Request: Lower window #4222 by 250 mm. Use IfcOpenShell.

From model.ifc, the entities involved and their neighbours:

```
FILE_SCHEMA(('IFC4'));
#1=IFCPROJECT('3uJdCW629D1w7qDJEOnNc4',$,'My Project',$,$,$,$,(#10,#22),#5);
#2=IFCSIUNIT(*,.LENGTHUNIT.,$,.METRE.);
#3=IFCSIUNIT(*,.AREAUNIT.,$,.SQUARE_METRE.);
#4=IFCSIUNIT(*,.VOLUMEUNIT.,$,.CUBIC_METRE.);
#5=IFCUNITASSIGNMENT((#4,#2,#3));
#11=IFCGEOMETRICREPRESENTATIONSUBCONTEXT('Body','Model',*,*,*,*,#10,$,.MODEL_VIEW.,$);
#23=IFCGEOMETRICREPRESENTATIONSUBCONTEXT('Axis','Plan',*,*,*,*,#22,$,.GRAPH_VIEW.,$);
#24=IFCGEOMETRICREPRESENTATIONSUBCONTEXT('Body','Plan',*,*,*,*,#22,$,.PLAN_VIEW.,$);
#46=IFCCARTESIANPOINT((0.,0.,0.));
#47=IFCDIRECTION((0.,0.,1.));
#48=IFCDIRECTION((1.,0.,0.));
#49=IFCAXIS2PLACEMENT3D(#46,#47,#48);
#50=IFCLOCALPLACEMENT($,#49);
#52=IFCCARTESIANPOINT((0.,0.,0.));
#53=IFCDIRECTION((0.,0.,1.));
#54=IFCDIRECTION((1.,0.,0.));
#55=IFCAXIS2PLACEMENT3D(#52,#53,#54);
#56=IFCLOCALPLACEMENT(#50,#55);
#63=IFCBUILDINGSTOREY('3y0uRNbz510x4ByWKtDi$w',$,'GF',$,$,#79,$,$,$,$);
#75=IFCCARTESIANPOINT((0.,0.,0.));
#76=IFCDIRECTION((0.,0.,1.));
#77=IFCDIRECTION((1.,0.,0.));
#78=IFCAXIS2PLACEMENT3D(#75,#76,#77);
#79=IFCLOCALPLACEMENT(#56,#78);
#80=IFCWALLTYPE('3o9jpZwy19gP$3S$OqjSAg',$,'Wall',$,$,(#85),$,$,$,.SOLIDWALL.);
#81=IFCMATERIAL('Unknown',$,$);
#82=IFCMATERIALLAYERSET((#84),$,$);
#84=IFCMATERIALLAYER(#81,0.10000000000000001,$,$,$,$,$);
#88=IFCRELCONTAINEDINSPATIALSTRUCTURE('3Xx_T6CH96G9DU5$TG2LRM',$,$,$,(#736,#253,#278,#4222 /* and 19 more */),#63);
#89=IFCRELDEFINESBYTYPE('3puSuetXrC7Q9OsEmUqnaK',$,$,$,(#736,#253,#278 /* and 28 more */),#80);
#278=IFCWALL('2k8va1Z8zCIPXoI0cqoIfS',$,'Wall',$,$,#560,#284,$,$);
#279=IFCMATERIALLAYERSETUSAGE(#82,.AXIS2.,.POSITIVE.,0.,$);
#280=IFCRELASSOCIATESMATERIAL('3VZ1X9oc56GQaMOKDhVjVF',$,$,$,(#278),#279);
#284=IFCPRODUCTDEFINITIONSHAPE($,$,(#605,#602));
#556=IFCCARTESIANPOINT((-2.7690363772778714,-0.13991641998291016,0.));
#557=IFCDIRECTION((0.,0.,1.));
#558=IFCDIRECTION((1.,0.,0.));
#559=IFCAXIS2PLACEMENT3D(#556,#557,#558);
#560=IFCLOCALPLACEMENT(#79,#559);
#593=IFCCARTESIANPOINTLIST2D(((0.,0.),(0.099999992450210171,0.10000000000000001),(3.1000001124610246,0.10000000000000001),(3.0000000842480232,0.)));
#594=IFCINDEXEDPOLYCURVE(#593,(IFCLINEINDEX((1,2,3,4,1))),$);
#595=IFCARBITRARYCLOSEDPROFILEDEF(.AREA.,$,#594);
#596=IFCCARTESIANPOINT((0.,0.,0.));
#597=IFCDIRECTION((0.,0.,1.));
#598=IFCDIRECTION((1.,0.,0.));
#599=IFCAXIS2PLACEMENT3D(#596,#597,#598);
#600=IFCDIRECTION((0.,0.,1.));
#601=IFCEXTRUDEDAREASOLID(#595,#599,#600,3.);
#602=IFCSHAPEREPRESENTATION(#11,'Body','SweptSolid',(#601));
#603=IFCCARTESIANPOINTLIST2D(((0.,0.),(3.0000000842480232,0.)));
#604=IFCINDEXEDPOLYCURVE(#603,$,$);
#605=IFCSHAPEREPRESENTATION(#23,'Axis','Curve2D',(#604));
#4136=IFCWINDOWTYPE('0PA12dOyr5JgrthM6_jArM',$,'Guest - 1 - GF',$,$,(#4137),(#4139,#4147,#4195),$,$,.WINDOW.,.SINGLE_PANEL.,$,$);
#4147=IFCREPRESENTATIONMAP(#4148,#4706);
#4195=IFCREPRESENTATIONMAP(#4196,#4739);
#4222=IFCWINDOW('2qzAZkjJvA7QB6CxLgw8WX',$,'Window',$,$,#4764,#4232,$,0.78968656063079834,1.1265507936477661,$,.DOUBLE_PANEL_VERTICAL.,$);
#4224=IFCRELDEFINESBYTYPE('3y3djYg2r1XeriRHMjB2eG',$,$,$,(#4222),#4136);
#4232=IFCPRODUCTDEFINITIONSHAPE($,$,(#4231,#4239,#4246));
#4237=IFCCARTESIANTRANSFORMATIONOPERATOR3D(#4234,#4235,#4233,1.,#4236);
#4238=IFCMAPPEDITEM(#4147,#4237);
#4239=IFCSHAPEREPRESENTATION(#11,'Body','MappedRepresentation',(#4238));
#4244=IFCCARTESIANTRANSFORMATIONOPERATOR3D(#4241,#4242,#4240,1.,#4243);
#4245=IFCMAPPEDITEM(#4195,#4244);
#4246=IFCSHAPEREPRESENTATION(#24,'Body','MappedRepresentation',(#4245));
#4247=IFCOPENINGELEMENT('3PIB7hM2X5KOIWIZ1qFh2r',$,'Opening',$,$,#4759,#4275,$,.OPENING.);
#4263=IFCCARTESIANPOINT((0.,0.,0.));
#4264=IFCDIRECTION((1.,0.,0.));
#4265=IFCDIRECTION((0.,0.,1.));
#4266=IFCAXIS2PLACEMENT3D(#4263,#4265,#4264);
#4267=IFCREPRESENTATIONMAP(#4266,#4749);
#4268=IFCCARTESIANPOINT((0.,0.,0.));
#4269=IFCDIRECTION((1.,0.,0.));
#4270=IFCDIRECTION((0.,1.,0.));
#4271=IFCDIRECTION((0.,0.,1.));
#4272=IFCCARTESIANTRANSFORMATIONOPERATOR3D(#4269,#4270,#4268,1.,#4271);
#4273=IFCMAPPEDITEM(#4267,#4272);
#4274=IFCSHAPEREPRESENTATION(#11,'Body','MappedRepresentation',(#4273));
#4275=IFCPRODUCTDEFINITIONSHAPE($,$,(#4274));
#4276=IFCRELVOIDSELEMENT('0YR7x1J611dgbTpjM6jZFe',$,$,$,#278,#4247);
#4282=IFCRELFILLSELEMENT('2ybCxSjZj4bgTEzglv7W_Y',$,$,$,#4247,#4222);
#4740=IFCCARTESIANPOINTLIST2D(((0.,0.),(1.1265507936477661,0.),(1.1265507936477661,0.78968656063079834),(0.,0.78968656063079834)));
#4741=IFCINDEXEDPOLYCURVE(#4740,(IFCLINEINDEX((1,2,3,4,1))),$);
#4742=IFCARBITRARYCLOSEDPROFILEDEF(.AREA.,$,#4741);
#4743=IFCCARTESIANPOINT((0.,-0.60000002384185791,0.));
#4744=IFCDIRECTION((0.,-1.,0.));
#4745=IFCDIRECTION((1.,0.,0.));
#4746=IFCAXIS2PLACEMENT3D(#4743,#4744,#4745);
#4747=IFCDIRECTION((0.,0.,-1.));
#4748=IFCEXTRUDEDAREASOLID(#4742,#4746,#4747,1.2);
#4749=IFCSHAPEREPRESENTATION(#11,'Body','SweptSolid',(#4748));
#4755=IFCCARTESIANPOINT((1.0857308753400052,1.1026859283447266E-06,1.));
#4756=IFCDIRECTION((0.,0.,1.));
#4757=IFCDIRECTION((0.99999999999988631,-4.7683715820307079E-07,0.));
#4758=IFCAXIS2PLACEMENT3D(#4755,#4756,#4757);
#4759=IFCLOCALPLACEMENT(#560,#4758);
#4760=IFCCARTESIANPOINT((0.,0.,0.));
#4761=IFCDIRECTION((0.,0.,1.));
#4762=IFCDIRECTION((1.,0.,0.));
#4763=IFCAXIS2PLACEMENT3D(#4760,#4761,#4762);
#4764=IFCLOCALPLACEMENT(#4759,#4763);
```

```python
import numpy as np
import ifcopenshell
import ifcopenshell.api.geometry
import ifcopenshell.util.placement
import ifcopenshell.util.unit

model = ifcopenshell.open("model.ifc")
unit_scale = ifcopenshell.util.unit.calculate_unit_scale(model)

window = model.by_id(4222)
opening = window.FillsVoids[0].RelatingOpeningElement
dz = -0.25 / unit_scale

shift = np.array([0.0, 0.0, dz])
# The window is placed relative to its opening, so it follows when the opening moves.
matrix = ifcopenshell.util.placement.get_local_placement(opening.ObjectPlacement)
matrix[:3, 3] += shift
ifcopenshell.api.geometry.edit_object_placement(
    model, product=opening, matrix=matrix, is_si=False, should_transform_children=True
)

print(f"moved by {dz * unit_scale:+.3f} m")

model.write("model_updated.ifc")
```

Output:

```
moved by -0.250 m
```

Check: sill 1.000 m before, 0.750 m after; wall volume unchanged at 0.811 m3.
